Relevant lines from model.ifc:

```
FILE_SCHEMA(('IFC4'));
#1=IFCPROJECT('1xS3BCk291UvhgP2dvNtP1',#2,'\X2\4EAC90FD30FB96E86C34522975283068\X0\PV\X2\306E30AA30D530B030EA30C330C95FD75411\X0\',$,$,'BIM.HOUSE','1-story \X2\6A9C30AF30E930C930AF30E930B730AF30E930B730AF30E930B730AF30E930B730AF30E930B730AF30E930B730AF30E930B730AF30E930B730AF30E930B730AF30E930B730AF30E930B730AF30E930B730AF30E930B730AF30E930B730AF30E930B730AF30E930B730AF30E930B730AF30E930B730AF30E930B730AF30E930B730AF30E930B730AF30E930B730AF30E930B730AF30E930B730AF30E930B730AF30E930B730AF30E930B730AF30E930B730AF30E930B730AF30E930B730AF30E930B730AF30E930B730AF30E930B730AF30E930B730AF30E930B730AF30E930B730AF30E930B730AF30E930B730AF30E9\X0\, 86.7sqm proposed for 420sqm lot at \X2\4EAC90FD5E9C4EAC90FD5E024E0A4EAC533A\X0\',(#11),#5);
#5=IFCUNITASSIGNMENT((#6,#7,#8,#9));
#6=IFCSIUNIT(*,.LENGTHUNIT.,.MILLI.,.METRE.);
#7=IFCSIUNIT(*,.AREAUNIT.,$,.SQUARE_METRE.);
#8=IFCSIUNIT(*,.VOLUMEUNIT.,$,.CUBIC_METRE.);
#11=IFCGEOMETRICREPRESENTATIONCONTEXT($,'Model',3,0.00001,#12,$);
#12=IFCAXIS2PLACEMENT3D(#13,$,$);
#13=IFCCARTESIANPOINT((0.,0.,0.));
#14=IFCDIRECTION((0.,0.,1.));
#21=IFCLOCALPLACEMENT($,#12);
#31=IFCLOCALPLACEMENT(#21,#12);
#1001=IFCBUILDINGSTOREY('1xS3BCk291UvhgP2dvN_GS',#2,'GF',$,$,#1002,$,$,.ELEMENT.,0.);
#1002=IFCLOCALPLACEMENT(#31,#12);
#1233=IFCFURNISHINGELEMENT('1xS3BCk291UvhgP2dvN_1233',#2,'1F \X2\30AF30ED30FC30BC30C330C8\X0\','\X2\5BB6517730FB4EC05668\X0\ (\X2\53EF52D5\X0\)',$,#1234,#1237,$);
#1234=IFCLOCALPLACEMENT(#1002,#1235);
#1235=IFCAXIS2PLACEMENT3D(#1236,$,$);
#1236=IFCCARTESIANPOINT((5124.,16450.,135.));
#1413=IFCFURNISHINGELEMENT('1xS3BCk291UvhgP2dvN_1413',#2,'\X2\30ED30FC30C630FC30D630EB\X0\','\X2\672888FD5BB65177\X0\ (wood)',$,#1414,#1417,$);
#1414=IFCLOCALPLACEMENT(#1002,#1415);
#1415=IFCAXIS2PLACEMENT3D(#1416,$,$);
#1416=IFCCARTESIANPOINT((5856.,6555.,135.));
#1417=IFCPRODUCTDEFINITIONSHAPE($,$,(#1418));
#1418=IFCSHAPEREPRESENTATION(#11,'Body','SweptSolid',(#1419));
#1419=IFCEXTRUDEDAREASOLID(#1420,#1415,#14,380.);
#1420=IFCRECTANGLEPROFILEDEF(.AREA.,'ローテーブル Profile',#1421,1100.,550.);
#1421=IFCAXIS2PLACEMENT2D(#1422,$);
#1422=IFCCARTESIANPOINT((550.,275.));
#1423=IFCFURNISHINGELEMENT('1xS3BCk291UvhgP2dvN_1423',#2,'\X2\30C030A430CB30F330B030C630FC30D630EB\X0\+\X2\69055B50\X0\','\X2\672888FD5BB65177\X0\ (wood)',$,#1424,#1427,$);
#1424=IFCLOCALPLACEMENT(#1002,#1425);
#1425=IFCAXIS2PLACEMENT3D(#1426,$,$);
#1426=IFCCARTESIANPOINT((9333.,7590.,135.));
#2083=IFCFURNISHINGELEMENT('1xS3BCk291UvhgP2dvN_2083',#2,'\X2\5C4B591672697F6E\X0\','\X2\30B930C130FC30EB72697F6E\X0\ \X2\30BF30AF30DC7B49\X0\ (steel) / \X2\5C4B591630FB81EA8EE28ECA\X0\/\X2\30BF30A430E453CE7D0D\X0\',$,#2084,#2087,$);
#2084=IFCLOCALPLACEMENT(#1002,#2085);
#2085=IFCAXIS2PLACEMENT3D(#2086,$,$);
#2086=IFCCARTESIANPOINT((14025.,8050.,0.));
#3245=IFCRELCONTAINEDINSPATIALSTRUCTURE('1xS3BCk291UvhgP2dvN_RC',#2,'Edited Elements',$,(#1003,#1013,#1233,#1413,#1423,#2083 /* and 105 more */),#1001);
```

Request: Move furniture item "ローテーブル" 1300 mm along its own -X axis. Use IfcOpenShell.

```python
import ifcopenshell
import ifcopenshell.api.geometry
import ifcopenshell.util.placement
import ifcopenshell.util.unit

model = ifcopenshell.open("model.ifc")
unit_scale = ifcopenshell.util.unit.calculate_unit_scale(model)

item = model.by_guid("1xS3BCk291UvhgP2dvN_1413")
matrix = ifcopenshell.util.placement.get_local_placement(item.ObjectPlacement)
matrix[:3, 3] -= matrix[:3, 0] * 1.3 / unit_scale
ifcopenshell.api.geometry.edit_object_placement(model, product=item, matrix=matrix, is_si=False)

print(ifcopenshell.util.placement.get_local_placement(item.ObjectPlacement).round(3) + 0.0)

model.write("model_rev.ifc")
```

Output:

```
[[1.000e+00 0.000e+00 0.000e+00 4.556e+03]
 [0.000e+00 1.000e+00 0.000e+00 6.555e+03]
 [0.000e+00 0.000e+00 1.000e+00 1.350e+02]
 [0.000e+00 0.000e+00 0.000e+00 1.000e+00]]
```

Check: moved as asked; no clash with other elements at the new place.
